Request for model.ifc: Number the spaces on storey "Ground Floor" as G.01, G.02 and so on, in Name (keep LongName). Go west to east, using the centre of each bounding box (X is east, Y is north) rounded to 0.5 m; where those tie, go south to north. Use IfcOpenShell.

First a look at what the model holds.

```python
import ifcopenshell
import ifcopenshell.util.element
import ifcopenshell.util.placement

model = ifcopenshell.open("model.ifc")
print(model.schema)
storey = next(s for s in model.by_type("IfcBuildingStorey") if s.Name == "Ground Floor")
spaces = [e for e in ifcopenshell.util.element.get_decomposition(storey) if e.is_a("IfcSpace")]
for e in sorted(spaces, key=lambda e: e.id()):
    origin = ifcopenshell.util.placement.get_local_placement(e.ObjectPlacement)[:3, 3]
    print(e.id(), e.Name, e.LongName, origin.round(2) + 0.0, sep=" | ")
```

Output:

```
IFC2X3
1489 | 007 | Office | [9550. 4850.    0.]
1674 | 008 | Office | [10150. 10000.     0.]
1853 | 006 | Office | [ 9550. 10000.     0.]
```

```python
import ifcopenshell
import ifcopenshell.geom
import ifcopenshell.util.element
import ifcopenshell.util.shape

model = ifcopenshell.open("model.ifc")
settings = ifcopenshell.geom.settings()
settings.set("use-world-coords", True)


def centre(element):
    shape = ifcopenshell.geom.create_shape(settings, element)
    return ifcopenshell.util.shape.get_bbox_centroid(shape.geometry)


storey = next(s for s in model.by_type("IfcBuildingStorey") if s.Name == "Ground Floor")
spaces = [e for e in ifcopenshell.util.element.get_decomposition(storey) if e.is_a("IfcSpace")]

# Insertion points can sit at a corner or the storey origin, so sort by the geometry (in metres).
centres = {e: centre(e) for e in spaces}
spaces.sort(key=lambda e: (round(centres[e][0] / 0.5), centres[e][1]))

for i, e in enumerate(spaces, start=1):
    number = f"G.{i:02d}"
    e.Name = number
    print(e.id(), number)

model.write("model_v2.ifc")
```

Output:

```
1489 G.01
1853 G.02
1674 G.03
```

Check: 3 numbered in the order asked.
